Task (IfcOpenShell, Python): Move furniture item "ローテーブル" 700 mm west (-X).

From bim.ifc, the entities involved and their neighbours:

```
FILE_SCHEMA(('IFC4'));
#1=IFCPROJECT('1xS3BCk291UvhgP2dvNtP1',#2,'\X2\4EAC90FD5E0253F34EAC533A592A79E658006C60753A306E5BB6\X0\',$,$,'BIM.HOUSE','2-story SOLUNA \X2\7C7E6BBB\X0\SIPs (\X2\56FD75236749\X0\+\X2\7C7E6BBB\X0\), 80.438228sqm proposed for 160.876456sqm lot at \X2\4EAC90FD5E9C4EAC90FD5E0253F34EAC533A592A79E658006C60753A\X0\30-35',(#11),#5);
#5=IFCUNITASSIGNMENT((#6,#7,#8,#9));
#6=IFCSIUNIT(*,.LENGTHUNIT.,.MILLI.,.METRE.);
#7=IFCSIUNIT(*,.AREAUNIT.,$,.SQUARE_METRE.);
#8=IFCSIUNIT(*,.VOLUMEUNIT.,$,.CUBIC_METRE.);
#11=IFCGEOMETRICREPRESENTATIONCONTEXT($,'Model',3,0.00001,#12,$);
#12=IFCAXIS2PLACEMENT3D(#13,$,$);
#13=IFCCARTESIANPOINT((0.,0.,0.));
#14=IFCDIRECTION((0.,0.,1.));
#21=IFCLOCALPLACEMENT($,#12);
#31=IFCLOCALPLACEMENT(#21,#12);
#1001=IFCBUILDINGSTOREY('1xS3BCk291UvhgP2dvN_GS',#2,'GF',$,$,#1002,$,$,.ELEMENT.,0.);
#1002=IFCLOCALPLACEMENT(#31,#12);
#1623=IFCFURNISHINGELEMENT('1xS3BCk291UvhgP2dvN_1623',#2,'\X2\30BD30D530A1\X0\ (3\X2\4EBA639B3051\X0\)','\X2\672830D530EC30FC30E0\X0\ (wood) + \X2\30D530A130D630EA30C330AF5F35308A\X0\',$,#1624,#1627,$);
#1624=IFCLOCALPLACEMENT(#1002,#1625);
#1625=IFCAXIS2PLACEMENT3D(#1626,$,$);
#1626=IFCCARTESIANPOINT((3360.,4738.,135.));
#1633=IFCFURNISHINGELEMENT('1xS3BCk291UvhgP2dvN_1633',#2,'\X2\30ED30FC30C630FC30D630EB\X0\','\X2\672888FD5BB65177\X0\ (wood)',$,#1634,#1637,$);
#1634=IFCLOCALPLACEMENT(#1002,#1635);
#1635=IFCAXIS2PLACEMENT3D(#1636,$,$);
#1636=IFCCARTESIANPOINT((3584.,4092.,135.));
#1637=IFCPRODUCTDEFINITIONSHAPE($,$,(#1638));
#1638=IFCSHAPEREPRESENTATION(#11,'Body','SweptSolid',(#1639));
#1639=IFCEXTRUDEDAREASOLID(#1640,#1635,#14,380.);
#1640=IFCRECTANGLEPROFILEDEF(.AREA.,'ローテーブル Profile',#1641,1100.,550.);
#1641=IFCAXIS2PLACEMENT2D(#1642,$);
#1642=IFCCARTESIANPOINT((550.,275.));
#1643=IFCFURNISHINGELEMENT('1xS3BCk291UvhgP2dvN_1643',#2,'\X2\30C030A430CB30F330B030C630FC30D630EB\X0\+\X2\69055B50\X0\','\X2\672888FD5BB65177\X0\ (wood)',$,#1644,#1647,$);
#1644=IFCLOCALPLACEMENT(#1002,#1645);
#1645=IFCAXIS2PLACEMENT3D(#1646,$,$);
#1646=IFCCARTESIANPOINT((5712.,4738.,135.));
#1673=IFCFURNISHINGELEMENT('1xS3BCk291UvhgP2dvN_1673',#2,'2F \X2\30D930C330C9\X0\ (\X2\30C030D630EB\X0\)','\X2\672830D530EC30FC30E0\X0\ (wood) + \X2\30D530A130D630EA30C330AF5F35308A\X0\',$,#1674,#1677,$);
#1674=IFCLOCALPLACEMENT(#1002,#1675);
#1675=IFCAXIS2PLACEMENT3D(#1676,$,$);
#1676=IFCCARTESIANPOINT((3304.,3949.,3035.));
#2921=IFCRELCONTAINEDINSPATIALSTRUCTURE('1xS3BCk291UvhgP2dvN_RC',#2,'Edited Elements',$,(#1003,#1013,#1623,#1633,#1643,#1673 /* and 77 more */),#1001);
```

```python
import ifcopenshell
import ifcopenshell.api.geometry
import ifcopenshell.util.placement

model = ifcopenshell.open("bim.ifc")

item = model.by_guid("1xS3BCk291UvhgP2dvN_1633")
matrix = ifcopenshell.util.placement.get_local_placement(item.ObjectPlacement)
matrix[0, 3] -= 700.0
ifcopenshell.api.geometry.edit_object_placement(model, product=item, matrix=matrix, is_si=False)

print(ifcopenshell.util.placement.get_local_placement(item.ObjectPlacement).round(3) + 0.0)

model.write("bim_v2.ifc")
```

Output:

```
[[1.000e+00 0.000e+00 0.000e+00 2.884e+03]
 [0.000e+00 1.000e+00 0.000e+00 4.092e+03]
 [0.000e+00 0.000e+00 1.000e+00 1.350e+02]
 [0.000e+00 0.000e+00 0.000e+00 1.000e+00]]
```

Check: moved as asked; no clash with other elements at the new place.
